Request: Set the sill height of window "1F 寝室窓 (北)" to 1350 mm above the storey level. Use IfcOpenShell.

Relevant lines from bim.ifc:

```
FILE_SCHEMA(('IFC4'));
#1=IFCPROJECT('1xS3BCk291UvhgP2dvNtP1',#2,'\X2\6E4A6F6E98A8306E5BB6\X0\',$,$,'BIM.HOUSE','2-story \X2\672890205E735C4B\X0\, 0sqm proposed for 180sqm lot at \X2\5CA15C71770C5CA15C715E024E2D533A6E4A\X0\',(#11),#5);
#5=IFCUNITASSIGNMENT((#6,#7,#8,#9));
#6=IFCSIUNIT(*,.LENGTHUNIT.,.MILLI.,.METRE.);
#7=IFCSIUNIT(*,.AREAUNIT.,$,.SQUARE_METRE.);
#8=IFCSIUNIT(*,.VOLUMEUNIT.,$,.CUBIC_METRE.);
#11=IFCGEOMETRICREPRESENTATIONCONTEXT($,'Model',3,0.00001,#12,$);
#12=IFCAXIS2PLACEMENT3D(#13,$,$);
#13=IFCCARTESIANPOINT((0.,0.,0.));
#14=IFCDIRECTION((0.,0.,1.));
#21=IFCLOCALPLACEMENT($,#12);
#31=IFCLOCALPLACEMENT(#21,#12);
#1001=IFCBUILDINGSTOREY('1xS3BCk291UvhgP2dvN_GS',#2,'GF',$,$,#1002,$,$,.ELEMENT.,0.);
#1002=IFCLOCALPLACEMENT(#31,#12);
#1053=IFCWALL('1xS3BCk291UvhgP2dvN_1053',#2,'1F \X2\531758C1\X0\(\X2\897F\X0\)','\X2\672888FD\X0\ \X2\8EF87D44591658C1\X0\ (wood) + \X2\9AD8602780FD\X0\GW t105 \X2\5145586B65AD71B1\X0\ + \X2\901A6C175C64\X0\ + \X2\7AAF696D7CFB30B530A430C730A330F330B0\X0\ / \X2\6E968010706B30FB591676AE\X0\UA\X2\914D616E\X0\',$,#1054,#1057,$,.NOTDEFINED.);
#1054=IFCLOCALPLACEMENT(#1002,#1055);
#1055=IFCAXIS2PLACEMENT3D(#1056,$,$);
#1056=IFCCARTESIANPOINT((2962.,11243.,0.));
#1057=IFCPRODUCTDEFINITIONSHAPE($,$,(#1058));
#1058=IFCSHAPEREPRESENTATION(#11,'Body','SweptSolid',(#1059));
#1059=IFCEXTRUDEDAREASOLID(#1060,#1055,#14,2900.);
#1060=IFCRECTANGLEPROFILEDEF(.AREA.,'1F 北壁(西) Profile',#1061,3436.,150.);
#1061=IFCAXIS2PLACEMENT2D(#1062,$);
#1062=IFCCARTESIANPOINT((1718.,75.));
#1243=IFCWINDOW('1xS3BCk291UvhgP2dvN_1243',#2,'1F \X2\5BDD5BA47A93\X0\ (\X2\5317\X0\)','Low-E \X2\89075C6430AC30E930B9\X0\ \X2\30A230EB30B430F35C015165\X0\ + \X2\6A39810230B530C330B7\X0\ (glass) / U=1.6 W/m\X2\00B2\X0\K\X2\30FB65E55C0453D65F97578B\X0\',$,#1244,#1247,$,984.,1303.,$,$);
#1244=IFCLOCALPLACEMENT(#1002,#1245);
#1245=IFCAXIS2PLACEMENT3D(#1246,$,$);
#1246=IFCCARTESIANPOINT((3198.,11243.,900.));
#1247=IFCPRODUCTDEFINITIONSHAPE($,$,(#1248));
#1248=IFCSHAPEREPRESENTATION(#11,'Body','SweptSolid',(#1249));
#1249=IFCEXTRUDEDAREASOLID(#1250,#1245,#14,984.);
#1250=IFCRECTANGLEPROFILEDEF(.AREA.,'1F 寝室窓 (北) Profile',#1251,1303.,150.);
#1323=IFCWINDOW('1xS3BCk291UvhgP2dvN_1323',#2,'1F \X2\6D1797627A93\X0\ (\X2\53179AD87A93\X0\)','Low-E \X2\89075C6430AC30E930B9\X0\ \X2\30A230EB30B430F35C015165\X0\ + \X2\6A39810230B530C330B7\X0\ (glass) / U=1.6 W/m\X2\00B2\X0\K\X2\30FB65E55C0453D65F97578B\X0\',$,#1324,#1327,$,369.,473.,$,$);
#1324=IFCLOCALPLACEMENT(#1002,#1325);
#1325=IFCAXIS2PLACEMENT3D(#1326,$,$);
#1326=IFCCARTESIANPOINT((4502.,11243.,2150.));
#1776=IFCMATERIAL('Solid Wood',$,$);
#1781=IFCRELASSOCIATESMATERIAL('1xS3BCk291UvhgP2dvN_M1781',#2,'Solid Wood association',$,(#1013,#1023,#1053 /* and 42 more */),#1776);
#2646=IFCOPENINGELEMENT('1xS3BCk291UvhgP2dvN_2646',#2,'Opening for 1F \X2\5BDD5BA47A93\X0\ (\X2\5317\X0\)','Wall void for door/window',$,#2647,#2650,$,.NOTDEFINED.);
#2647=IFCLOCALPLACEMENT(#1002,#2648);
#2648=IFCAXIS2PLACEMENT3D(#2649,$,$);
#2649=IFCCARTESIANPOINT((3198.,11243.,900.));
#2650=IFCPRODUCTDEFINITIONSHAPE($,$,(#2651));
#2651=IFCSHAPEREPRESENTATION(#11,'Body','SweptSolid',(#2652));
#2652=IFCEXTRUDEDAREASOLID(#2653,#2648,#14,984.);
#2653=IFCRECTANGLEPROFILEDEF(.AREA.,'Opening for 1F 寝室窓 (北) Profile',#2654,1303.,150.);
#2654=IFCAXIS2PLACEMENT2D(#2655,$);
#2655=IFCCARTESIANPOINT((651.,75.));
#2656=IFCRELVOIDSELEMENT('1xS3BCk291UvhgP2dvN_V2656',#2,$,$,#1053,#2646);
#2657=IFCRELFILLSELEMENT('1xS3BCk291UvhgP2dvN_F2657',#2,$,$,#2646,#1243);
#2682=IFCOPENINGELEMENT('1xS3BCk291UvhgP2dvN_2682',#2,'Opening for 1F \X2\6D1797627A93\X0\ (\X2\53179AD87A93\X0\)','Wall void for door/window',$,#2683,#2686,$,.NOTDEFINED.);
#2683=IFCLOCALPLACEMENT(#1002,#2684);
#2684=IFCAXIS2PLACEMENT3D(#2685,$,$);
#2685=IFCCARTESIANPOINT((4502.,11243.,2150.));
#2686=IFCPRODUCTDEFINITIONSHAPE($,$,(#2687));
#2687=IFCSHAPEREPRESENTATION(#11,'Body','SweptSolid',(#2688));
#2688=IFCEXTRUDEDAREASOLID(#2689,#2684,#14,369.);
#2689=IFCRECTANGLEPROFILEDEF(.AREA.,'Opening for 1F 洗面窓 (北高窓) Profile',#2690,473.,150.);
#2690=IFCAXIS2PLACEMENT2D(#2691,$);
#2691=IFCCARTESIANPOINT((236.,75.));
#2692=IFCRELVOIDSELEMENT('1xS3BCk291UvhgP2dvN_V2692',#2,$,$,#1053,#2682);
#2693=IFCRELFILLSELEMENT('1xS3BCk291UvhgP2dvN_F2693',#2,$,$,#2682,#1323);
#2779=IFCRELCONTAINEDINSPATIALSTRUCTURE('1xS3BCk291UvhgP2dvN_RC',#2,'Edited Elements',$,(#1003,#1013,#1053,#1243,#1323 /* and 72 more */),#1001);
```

```python
import numpy as np
import ifcopenshell
import ifcopenshell.api.geometry
import ifcopenshell.geom
import ifcopenshell.util.element
import ifcopenshell.util.placement
import ifcopenshell.util.shape
import ifcopenshell.util.unit

model = ifcopenshell.open("bim.ifc")
unit_scale = ifcopenshell.util.unit.calculate_unit_scale(model)

window = model.by_guid("1xS3BCk291UvhgP2dvN_1243")
opening = window.FillsVoids[0].RelatingOpeningElement
storey = ifcopenshell.util.element.get_container(window, ifc_class="IfcBuildingStorey")
level = ifcopenshell.util.placement.get_local_placement(storey.ObjectPlacement)[2, 3]

# The opening's origin need not be at the sill, so measure its lowest point.
shape = ifcopenshell.geom.create_shape(ifcopenshell.geom.settings(), opening)
bottom = ifcopenshell.util.shape.get_shape_bottom_elevation(shape, shape.geometry) / unit_scale
dz = level + 1.35 / unit_scale - bottom

shift = np.array([0.0, 0.0, dz])
# The window is not placed relative to its opening, so move both.
for product in (opening, window):
    matrix = ifcopenshell.util.placement.get_local_placement(product.ObjectPlacement)
    matrix[:3, 3] += shift
    ifcopenshell.api.geometry.edit_object_placement(model, product=product, matrix=matrix, is_si=False)

print(f"moved by {dz * unit_scale:+.3f} m")

model.write("bim-out.ifc")
```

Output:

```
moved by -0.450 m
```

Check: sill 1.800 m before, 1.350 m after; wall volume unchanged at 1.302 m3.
